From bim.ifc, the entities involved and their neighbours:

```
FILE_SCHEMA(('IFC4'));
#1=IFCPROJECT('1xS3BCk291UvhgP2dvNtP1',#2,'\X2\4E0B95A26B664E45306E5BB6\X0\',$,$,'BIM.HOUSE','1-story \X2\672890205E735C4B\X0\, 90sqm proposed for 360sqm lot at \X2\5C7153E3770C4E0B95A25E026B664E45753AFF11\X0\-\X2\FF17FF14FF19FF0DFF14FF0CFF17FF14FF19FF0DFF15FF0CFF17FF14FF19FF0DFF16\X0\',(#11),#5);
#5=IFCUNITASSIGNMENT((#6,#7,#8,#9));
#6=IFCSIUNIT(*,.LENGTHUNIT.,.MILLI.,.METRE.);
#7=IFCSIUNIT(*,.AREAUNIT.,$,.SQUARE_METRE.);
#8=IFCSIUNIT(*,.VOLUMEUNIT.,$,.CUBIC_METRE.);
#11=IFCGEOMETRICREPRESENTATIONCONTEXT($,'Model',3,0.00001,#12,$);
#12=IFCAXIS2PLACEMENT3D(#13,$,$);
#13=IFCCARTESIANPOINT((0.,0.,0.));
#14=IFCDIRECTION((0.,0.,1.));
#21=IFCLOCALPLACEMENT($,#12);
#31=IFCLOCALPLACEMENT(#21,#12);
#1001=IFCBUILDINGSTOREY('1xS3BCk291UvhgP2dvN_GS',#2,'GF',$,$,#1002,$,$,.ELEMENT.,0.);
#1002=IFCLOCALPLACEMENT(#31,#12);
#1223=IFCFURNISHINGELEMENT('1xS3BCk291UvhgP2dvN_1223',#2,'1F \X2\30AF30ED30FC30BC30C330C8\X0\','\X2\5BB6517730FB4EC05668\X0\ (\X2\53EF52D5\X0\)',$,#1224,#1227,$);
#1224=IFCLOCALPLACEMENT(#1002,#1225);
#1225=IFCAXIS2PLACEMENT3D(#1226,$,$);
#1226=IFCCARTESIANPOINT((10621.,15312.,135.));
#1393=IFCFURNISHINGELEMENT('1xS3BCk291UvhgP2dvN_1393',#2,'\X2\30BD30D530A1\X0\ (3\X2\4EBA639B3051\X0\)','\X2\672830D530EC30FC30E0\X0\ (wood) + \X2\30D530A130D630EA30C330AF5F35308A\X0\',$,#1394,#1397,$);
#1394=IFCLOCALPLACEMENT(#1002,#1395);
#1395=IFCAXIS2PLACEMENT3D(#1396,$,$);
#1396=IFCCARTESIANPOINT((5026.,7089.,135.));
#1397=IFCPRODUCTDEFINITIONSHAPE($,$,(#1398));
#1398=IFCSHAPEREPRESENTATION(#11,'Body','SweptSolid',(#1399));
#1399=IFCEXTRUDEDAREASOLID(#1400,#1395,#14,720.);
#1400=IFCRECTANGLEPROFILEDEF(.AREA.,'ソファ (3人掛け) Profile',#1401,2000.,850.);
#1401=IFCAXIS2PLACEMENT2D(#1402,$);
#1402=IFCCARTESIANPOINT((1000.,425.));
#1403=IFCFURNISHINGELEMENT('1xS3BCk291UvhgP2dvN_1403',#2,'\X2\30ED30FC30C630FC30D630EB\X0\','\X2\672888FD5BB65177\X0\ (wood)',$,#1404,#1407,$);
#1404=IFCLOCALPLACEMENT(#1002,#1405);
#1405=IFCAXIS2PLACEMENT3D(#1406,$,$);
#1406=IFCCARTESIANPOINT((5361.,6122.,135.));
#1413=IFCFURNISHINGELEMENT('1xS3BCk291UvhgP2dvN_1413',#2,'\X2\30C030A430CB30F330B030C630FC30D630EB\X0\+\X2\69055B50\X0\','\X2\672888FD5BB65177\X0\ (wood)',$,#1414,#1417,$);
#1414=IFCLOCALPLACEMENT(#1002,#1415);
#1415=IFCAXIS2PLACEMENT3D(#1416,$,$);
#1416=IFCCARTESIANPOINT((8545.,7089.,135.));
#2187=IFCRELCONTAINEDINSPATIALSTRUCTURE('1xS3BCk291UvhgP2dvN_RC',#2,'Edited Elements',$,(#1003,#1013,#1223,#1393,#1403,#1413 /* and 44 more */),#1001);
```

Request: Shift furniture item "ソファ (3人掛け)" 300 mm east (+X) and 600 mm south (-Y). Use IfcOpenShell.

```python
import ifcopenshell
import ifcopenshell.api.geometry
import ifcopenshell.util.placement

model = ifcopenshell.open("bim.ifc")

item = model.by_guid("1xS3BCk291UvhgP2dvN_1393")
matrix = ifcopenshell.util.placement.get_local_placement(item.ObjectPlacement)
matrix[0, 3] += 300.0
matrix[1, 3] -= 600.0
ifcopenshell.api.geometry.edit_object_placement(model, product=item, matrix=matrix, is_si=False)

print(ifcopenshell.util.placement.get_local_placement(item.ObjectPlacement).round(3) + 0.0)

model.write("bim_v2.ifc")
```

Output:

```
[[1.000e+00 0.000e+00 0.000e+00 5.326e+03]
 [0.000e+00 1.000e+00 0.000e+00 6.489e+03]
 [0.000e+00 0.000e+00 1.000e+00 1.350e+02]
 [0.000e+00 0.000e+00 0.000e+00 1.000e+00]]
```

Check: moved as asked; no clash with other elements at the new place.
